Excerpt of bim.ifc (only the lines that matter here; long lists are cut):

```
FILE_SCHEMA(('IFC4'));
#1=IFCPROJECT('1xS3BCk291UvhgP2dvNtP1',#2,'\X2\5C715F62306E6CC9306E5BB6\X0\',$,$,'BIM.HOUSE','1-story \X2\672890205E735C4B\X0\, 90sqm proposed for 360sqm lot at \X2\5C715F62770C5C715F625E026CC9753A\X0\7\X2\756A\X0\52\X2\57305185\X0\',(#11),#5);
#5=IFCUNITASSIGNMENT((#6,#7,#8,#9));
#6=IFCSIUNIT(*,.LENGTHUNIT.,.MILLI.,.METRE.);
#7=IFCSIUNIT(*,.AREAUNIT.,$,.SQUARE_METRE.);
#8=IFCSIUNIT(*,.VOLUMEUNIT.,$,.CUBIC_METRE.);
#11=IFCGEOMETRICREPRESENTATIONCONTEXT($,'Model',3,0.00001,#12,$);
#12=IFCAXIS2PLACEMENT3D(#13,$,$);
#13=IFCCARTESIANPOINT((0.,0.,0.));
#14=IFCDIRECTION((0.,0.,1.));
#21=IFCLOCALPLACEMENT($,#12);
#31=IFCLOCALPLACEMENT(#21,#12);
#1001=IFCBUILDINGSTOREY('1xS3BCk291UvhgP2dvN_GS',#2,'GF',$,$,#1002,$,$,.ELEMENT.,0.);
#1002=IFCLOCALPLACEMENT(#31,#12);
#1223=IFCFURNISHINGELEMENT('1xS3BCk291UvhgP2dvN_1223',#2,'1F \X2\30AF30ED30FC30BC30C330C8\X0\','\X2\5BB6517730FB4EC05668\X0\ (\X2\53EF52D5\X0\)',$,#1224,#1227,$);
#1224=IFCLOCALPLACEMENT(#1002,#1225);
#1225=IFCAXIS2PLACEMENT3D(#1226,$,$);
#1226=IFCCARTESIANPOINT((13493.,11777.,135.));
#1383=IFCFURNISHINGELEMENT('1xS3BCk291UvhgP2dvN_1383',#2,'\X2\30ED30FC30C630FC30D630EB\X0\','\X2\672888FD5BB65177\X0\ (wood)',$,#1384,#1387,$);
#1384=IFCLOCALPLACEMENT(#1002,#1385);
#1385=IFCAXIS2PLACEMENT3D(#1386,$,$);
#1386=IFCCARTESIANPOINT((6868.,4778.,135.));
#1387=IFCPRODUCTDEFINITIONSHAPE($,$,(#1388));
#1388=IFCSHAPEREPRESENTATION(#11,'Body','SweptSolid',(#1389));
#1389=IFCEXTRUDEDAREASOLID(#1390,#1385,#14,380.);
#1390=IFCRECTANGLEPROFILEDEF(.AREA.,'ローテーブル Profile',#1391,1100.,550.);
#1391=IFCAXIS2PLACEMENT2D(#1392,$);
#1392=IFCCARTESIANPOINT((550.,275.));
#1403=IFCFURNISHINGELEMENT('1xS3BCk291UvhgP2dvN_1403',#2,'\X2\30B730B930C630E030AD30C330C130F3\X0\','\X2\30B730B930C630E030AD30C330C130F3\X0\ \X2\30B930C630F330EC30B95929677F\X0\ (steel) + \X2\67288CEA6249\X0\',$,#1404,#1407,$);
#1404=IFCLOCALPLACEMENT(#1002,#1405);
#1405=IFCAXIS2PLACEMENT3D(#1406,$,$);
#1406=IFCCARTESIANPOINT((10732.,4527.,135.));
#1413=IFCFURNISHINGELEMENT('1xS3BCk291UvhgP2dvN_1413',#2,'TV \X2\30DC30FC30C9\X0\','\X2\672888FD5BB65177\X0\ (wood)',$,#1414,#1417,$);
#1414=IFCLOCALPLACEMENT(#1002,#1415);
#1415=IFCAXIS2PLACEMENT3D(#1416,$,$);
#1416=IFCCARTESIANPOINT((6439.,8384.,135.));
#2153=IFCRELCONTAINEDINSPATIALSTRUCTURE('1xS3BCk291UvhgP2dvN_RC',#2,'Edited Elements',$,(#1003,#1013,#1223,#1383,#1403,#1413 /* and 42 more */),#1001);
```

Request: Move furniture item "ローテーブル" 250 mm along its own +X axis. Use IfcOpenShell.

```python
import ifcopenshell
import ifcopenshell.api.geometry
import ifcopenshell.util.placement
import ifcopenshell.util.unit

model = ifcopenshell.open("bim.ifc")
unit_scale = ifcopenshell.util.unit.calculate_unit_scale(model)

item = model.by_guid("1xS3BCk291UvhgP2dvN_1383")
matrix = ifcopenshell.util.placement.get_local_placement(item.ObjectPlacement)
matrix[:3, 3] += matrix[:3, 0] * 0.25 / unit_scale
ifcopenshell.api.geometry.edit_object_placement(model, product=item, matrix=matrix, is_si=False)

print(ifcopenshell.util.placement.get_local_placement(item.ObjectPlacement).round(3) + 0.0)

model.write("bim-out.ifc")
```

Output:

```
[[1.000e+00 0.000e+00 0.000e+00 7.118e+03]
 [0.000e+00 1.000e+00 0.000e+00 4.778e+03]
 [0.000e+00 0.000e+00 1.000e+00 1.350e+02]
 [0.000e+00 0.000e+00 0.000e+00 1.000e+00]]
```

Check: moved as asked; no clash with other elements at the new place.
